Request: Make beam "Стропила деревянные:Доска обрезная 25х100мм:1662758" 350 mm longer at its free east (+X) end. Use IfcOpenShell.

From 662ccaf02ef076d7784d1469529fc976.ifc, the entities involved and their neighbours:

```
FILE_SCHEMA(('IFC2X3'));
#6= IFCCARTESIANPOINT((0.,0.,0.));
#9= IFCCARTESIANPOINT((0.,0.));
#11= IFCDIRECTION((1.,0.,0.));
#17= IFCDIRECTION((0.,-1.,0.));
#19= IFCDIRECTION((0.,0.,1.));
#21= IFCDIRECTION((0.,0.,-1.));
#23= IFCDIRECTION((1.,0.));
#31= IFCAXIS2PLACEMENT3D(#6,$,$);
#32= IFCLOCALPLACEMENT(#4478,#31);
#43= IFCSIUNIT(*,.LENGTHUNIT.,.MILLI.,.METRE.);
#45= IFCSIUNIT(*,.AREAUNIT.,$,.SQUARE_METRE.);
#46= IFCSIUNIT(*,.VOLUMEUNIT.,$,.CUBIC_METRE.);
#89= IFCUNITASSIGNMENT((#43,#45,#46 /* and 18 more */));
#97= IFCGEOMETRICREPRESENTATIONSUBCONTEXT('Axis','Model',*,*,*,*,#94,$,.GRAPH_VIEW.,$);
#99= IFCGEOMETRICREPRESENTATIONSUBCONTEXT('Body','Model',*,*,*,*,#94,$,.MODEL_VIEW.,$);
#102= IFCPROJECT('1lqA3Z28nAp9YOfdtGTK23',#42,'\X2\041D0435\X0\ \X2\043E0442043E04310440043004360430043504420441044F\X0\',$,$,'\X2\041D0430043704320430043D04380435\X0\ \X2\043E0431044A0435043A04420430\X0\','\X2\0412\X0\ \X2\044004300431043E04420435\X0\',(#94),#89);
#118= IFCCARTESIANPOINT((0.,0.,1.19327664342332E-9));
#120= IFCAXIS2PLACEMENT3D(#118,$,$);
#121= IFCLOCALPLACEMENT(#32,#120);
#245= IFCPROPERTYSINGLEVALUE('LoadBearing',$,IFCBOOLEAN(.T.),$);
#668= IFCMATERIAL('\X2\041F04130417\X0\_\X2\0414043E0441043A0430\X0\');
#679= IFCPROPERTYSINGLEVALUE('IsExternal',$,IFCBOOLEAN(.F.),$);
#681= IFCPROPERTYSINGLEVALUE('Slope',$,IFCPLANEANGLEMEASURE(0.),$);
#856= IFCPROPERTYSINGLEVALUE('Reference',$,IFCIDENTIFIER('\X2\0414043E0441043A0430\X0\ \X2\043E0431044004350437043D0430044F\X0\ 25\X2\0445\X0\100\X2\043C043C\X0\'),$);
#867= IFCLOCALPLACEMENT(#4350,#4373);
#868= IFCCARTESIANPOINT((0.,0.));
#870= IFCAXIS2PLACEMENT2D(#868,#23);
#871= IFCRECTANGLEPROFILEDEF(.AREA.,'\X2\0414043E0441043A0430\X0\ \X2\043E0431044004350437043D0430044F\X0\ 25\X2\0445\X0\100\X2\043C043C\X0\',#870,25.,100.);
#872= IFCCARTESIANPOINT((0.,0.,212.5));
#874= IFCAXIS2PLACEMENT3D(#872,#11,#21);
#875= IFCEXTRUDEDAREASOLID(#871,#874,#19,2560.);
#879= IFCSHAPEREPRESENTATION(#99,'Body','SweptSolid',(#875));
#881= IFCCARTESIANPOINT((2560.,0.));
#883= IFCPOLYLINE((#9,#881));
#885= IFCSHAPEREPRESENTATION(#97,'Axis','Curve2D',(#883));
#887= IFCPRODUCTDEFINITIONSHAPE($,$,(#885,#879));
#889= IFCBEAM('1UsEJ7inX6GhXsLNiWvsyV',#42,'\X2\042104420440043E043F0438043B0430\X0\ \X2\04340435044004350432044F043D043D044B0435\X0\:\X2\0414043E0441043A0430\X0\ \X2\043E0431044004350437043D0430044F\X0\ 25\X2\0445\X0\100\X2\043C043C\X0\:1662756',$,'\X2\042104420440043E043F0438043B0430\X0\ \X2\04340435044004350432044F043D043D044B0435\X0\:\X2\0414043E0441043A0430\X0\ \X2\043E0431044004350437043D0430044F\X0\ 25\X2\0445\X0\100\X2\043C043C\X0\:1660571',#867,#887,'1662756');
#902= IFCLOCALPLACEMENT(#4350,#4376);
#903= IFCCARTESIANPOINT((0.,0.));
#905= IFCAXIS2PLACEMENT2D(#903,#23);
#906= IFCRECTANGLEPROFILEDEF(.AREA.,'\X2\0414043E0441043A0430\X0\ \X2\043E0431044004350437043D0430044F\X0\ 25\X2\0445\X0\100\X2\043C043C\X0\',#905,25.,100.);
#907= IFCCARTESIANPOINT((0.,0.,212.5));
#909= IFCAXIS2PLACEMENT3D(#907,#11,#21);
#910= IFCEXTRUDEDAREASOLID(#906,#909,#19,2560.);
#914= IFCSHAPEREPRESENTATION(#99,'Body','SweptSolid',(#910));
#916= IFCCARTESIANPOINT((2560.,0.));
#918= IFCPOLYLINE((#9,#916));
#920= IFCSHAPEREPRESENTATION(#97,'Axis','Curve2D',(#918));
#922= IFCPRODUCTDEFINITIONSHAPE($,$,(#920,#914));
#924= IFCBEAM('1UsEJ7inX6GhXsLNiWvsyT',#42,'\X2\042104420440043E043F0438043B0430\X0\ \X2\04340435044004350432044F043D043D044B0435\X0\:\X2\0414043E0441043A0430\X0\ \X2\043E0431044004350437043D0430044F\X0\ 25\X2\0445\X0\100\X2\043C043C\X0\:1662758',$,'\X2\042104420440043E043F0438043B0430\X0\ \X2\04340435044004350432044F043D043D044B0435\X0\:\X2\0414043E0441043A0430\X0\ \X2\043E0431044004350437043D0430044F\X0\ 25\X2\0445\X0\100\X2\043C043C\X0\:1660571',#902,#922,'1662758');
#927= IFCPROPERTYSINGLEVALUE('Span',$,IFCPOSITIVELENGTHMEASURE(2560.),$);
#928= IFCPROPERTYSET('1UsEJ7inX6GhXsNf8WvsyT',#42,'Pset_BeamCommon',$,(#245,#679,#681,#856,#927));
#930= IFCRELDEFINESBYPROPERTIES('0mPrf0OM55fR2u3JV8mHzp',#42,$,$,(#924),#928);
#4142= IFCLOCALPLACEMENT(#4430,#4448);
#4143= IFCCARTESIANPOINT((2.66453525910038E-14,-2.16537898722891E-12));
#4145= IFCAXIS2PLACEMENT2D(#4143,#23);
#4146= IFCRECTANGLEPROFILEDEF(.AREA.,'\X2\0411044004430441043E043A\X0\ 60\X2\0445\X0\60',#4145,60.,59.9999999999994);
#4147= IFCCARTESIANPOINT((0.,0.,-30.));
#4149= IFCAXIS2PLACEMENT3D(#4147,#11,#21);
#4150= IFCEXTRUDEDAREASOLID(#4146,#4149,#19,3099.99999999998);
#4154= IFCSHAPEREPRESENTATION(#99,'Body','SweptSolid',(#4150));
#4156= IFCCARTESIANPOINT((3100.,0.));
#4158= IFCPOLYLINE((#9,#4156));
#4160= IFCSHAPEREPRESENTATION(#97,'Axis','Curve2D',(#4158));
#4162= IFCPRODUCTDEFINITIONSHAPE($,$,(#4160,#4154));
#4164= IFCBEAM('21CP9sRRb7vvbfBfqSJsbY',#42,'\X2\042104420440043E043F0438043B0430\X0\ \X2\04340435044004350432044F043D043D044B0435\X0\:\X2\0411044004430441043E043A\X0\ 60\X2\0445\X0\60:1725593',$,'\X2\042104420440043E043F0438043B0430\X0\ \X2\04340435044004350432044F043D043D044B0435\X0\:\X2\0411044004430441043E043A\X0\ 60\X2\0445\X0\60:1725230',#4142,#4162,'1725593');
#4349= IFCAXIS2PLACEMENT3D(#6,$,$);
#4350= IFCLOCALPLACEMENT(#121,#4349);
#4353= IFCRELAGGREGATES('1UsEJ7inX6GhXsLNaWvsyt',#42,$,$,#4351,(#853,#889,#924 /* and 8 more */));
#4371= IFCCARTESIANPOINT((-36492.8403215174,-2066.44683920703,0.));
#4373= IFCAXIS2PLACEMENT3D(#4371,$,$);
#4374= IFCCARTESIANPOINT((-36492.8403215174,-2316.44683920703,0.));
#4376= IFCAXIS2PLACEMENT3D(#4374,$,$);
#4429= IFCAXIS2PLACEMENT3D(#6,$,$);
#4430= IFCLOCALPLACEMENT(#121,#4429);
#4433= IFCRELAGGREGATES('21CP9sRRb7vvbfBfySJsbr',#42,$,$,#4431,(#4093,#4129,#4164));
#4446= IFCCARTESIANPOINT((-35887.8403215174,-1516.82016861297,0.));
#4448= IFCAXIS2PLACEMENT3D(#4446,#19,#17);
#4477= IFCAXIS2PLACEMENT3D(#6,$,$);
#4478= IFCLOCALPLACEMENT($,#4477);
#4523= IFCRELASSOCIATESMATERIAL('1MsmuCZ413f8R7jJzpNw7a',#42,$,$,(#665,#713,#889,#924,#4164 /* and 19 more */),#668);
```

```python
import numpy as np
import ifcopenshell
import ifcopenshell.api.pset
import ifcopenshell.util.element
import ifcopenshell.util.representation
import ifcopenshell.util.unit

model = ifcopenshell.open("662ccaf02ef076d7784d1469529fc976.ifc")
unit_scale = ifcopenshell.util.unit.calculate_unit_scale(model)

member = model.by_id(924)
change = 0.35 / unit_scale

# The extrusion runs towards the end named, so only its depth changes.
body = ifcopenshell.util.representation.get_representation(member, "Model", "Body")
solid = body.Items[0]
old_length = solid.Depth
solid.Depth += change

# Move the axis end point with it.
axis = next(r for r in member.Representation.Representations if r.RepresentationIdentifier == "Axis").Items[0]
start, end = (np.array(p.Coordinates) for p in axis.Points)
end = end + (end - start) / np.linalg.norm(end - start) * change
point = model.createIfcCartesianPoint(end.tolist())
axis.Points = [axis.Points[0], point]

# Update the stored length and volume.
pset = model.by_id(ifcopenshell.util.element.get_pset(member, "Pset_BeamCommon", should_inherit=False)["id"])
ifcopenshell.api.pset.edit_pset(model, pset=pset, properties={
    "Span": model.create_entity("IfcPositiveLengthMeasure", solid.Depth),
})

print(f"length {old_length:g} -> {solid.Depth:g}")

model.write("662ccaf02ef076d7784d1469529fc976_rev.ifc")
```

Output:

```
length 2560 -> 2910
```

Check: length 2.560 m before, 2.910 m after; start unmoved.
